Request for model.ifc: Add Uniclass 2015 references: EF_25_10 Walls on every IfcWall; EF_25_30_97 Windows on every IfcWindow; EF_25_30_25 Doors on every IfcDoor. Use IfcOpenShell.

First a look at what the model holds.

```python
import ifcopenshell

model = ifcopenshell.open("model.ifc")
print(model.schema)
print("classifications:", [c.Name for c in model.by_type("IfcClassification")])
for ifc_class in ("IfcDoor", "IfcRoof", "IfcStair", "IfcWall", "IfcWindow"):
    print(ifc_class, len(model.by_type(ifc_class)))
```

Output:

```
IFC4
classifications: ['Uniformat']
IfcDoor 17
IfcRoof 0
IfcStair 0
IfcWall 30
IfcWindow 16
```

```python
import ifcopenshell
import ifcopenshell.api.classification

model = ifcopenshell.open("model.ifc")

system = ifcopenshell.api.classification.add_classification(model, classification="Uniclass 2015")

codes = {
    "IfcWall": ("EF_25_10", "Walls"),
    "IfcWindow": ("EF_25_30_97", "Windows"),
    "IfcDoor": ("EF_25_30_25", "Doors"),
}
for ifc_class, (code, name) in codes.items():
    products = model.by_type(ifc_class)
    ifcopenshell.api.classification.add_reference(
        model, products=products, classification=system, identification=code, name=name
    )
    print(code, len(products))

model.write("model-out.ifc")
```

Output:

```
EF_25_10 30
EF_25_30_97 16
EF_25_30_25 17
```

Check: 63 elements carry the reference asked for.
